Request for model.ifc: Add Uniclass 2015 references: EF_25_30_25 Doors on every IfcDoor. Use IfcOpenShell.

First a look at what the model holds.

```python
import ifcopenshell

model = ifcopenshell.open("model.ifc")
print(model.schema)
print("classifications:", [c.Name for c in model.by_type("IfcClassification")])
for ifc_class in ("IfcDoor", "IfcRoof", "IfcStair", "IfcWall", "IfcWindow"):
    print(ifc_class, len(model.by_type(ifc_class)))
```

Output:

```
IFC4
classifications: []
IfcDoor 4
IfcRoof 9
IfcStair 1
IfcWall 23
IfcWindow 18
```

```python
import ifcopenshell
import ifcopenshell.api.classification

model = ifcopenshell.open("model.ifc")

system = ifcopenshell.api.classification.add_classification(model, classification="Uniclass 2015")

codes = {
    "IfcDoor": ("EF_25_30_25", "Doors"),
}
for ifc_class, (code, name) in codes.items():
    products = model.by_type(ifc_class)
    ifcopenshell.api.classification.add_reference(
        model, products=products, classification=system, identification=code, name=name
    )
    print(code, len(products))

model.write("model_rev.ifc")
```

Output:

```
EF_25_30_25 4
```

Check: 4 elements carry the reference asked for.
